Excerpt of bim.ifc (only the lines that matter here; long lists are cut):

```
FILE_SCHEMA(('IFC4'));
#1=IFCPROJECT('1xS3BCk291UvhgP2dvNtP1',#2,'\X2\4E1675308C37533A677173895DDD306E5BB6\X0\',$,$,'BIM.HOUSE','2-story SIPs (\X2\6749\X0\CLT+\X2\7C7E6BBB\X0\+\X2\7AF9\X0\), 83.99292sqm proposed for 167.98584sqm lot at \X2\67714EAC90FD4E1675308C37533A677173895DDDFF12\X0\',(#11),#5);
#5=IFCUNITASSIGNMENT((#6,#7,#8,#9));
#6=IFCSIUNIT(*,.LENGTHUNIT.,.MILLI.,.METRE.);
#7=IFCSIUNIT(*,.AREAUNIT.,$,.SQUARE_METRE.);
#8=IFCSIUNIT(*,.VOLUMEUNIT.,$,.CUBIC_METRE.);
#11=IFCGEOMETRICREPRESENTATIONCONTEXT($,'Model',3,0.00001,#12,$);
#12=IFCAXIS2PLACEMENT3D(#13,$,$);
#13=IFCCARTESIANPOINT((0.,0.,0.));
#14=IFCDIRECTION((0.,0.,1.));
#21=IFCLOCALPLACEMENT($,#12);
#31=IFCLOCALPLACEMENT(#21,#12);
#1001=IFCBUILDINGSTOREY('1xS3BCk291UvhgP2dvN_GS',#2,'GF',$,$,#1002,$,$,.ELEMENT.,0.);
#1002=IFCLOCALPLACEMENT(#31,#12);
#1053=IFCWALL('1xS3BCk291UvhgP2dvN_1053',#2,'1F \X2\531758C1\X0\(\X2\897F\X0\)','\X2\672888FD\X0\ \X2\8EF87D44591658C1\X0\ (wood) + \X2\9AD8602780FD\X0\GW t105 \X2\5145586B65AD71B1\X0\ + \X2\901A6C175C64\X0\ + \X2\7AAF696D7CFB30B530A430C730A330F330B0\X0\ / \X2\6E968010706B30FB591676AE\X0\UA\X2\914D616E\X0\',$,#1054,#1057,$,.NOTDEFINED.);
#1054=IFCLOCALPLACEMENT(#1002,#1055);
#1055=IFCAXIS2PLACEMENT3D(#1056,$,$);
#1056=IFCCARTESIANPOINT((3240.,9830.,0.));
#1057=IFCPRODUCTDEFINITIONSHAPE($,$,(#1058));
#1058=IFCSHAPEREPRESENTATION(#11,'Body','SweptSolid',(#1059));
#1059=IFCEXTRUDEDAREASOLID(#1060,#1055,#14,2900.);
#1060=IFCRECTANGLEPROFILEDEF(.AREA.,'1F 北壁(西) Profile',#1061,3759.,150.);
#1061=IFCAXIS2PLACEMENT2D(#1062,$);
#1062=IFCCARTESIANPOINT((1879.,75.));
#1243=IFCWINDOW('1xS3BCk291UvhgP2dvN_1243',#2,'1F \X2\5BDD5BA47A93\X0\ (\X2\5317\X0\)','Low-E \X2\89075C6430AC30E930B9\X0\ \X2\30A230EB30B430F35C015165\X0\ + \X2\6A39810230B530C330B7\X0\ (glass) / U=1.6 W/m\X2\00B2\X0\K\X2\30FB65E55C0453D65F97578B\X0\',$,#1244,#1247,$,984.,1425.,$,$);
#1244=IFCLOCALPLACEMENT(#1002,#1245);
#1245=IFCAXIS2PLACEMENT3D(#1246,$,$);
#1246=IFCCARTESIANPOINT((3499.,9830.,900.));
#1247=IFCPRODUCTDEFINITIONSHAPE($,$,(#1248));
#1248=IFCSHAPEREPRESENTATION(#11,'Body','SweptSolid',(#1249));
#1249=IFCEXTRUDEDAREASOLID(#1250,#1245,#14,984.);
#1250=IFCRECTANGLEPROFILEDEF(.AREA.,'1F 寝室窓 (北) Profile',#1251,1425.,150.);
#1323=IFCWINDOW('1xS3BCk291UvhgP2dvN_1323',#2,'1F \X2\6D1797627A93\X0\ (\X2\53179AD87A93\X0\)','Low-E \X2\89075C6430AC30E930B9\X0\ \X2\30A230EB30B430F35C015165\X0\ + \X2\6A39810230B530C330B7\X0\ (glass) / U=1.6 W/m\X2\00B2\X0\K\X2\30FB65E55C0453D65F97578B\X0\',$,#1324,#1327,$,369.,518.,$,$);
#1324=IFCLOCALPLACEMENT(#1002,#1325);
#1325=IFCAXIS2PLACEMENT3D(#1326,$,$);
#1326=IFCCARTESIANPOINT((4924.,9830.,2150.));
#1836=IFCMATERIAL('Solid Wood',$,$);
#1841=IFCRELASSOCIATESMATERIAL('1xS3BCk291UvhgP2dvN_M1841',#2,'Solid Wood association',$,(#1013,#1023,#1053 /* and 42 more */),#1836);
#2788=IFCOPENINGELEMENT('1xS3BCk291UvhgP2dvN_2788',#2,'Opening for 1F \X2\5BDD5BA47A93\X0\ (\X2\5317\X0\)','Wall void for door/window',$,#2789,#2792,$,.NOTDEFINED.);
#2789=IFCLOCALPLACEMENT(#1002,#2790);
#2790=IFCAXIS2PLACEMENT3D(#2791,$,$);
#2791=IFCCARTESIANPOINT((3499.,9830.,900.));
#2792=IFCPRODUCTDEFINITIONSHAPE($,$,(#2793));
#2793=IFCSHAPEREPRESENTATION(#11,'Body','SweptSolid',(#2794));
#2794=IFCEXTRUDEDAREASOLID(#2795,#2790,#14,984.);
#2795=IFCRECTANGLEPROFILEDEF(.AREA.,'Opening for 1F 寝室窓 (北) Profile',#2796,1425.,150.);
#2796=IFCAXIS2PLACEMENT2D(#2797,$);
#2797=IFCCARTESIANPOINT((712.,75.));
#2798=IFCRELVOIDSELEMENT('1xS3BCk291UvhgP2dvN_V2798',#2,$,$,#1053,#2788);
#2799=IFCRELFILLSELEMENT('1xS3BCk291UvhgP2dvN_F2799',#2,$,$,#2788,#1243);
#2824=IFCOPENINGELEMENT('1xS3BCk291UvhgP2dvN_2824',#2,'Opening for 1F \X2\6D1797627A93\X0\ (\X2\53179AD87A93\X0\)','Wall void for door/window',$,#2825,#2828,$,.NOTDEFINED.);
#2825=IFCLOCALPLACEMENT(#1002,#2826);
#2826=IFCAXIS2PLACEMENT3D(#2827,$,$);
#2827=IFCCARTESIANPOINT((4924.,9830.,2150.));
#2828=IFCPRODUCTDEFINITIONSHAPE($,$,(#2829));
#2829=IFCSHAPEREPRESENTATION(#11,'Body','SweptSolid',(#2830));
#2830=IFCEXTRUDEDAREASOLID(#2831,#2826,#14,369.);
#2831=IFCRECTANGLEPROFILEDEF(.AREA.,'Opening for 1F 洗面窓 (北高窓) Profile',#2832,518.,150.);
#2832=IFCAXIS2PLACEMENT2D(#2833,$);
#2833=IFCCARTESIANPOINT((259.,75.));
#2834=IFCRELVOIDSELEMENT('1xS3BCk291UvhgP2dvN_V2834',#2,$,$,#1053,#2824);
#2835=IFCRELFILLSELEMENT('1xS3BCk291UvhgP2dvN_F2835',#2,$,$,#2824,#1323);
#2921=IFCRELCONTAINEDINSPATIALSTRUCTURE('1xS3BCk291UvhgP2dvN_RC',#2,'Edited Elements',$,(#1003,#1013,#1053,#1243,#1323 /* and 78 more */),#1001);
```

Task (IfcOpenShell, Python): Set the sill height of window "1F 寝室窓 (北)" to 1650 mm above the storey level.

```python
import numpy as np
import ifcopenshell
import ifcopenshell.api.geometry
import ifcopenshell.geom
import ifcopenshell.util.element
import ifcopenshell.util.placement
import ifcopenshell.util.shape
import ifcopenshell.util.unit

model = ifcopenshell.open("bim.ifc")
unit_scale = ifcopenshell.util.unit.calculate_unit_scale(model)

window = model.by_guid("1xS3BCk291UvhgP2dvN_1243")
opening = window.FillsVoids[0].RelatingOpeningElement
storey = ifcopenshell.util.element.get_container(window, ifc_class="IfcBuildingStorey")
level = ifcopenshell.util.placement.get_local_placement(storey.ObjectPlacement)[2, 3]

# The opening's origin need not be at the sill, so measure its lowest point.
shape = ifcopenshell.geom.create_shape(ifcopenshell.geom.settings(), opening)
bottom = ifcopenshell.util.shape.get_shape_bottom_elevation(shape, shape.geometry) / unit_scale
dz = level + 1.65 / unit_scale - bottom

shift = np.array([0.0, 0.0, dz])
# The window is not placed relative to its opening, so move both.
for product in (opening, window):
    matrix = ifcopenshell.util.placement.get_local_placement(product.ObjectPlacement)
    matrix[:3, 3] += shift
    ifcopenshell.api.geometry.edit_object_placement(model, product=product, matrix=matrix, is_si=False)

print(f"moved by {dz * unit_scale:+.3f} m")

model.write("bim_edited.ifc")
```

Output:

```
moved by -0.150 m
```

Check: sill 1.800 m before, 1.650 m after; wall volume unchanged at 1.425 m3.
